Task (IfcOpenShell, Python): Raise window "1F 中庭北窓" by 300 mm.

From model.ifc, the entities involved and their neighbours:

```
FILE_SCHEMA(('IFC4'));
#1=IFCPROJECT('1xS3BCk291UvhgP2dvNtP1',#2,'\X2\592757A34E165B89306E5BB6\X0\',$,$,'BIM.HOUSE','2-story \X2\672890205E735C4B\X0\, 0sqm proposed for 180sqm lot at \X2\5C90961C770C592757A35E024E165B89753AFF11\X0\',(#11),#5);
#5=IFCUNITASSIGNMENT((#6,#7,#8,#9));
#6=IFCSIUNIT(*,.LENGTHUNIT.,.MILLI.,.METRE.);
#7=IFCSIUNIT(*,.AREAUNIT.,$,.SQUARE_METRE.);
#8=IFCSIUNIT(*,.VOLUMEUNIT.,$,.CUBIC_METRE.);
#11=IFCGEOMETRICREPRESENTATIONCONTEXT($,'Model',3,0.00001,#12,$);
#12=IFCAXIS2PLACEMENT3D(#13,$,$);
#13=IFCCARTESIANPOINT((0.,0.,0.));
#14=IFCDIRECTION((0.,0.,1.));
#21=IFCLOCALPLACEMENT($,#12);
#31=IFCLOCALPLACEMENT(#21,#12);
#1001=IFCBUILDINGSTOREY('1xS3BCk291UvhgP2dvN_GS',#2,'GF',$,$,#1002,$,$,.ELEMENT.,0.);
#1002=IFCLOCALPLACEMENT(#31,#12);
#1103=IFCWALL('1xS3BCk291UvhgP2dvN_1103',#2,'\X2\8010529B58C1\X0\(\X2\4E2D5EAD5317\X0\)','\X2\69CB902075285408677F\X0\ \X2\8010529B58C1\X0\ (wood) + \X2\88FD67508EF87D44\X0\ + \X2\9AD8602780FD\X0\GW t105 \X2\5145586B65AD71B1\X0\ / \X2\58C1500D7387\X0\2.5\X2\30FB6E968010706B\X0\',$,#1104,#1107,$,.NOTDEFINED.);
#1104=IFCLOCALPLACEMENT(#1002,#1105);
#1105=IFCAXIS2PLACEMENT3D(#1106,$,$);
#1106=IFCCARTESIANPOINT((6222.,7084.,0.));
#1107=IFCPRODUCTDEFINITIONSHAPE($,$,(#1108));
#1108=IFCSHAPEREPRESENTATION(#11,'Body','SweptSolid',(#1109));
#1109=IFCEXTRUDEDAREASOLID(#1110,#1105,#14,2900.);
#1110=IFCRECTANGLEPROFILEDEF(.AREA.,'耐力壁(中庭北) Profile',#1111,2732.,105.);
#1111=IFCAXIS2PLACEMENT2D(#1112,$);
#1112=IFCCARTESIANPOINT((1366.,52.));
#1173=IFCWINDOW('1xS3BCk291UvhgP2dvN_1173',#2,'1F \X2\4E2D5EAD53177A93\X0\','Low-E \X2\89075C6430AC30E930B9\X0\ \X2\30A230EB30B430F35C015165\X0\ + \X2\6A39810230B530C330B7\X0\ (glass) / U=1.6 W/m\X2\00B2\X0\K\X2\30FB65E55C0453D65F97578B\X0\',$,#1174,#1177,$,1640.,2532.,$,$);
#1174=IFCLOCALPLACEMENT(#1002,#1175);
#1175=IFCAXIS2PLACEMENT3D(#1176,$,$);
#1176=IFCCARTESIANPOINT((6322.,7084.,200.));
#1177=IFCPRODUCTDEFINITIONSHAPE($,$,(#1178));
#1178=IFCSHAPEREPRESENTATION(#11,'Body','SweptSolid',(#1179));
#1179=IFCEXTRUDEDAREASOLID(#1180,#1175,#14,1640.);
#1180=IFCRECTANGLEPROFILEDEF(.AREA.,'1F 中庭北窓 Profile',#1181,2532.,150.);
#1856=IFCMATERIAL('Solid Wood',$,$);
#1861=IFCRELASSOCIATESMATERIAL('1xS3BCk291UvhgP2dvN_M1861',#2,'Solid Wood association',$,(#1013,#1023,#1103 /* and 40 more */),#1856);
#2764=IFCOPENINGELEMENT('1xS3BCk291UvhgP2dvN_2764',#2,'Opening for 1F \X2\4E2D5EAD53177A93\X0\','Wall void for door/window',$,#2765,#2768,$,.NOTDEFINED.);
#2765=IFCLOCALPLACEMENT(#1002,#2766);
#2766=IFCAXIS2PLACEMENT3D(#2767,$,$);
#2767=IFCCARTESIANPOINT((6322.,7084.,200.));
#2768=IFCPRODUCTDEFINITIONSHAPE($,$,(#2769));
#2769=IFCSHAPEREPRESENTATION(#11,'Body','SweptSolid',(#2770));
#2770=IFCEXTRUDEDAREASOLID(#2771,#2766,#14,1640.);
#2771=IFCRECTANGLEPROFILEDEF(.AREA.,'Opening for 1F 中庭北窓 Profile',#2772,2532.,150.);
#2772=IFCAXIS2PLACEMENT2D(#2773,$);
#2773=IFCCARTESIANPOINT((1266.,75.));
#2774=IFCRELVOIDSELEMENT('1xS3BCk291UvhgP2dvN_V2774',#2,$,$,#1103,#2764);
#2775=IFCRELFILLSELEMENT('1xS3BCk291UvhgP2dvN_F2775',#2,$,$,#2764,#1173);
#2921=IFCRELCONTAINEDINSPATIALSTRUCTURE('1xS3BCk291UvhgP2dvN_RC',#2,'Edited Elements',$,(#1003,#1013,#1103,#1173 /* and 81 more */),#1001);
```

```python
import numpy as np
import ifcopenshell
import ifcopenshell.api.geometry
import ifcopenshell.util.placement
import ifcopenshell.util.unit

model = ifcopenshell.open("model.ifc")
unit_scale = ifcopenshell.util.unit.calculate_unit_scale(model)

window = model.by_guid("1xS3BCk291UvhgP2dvN_1173")
opening = window.FillsVoids[0].RelatingOpeningElement
dz = 300.0

shift = np.array([0.0, 0.0, dz])
# The window is not placed relative to its opening, so move both.
for product in (opening, window):
    matrix = ifcopenshell.util.placement.get_local_placement(product.ObjectPlacement)
    matrix[:3, 3] += shift
    ifcopenshell.api.geometry.edit_object_placement(model, product=product, matrix=matrix, is_si=False)

print(f"moved by {dz * unit_scale:+.3f} m")

model.write("model_v2.ifc")
```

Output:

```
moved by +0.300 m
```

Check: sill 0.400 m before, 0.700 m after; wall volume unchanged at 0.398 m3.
